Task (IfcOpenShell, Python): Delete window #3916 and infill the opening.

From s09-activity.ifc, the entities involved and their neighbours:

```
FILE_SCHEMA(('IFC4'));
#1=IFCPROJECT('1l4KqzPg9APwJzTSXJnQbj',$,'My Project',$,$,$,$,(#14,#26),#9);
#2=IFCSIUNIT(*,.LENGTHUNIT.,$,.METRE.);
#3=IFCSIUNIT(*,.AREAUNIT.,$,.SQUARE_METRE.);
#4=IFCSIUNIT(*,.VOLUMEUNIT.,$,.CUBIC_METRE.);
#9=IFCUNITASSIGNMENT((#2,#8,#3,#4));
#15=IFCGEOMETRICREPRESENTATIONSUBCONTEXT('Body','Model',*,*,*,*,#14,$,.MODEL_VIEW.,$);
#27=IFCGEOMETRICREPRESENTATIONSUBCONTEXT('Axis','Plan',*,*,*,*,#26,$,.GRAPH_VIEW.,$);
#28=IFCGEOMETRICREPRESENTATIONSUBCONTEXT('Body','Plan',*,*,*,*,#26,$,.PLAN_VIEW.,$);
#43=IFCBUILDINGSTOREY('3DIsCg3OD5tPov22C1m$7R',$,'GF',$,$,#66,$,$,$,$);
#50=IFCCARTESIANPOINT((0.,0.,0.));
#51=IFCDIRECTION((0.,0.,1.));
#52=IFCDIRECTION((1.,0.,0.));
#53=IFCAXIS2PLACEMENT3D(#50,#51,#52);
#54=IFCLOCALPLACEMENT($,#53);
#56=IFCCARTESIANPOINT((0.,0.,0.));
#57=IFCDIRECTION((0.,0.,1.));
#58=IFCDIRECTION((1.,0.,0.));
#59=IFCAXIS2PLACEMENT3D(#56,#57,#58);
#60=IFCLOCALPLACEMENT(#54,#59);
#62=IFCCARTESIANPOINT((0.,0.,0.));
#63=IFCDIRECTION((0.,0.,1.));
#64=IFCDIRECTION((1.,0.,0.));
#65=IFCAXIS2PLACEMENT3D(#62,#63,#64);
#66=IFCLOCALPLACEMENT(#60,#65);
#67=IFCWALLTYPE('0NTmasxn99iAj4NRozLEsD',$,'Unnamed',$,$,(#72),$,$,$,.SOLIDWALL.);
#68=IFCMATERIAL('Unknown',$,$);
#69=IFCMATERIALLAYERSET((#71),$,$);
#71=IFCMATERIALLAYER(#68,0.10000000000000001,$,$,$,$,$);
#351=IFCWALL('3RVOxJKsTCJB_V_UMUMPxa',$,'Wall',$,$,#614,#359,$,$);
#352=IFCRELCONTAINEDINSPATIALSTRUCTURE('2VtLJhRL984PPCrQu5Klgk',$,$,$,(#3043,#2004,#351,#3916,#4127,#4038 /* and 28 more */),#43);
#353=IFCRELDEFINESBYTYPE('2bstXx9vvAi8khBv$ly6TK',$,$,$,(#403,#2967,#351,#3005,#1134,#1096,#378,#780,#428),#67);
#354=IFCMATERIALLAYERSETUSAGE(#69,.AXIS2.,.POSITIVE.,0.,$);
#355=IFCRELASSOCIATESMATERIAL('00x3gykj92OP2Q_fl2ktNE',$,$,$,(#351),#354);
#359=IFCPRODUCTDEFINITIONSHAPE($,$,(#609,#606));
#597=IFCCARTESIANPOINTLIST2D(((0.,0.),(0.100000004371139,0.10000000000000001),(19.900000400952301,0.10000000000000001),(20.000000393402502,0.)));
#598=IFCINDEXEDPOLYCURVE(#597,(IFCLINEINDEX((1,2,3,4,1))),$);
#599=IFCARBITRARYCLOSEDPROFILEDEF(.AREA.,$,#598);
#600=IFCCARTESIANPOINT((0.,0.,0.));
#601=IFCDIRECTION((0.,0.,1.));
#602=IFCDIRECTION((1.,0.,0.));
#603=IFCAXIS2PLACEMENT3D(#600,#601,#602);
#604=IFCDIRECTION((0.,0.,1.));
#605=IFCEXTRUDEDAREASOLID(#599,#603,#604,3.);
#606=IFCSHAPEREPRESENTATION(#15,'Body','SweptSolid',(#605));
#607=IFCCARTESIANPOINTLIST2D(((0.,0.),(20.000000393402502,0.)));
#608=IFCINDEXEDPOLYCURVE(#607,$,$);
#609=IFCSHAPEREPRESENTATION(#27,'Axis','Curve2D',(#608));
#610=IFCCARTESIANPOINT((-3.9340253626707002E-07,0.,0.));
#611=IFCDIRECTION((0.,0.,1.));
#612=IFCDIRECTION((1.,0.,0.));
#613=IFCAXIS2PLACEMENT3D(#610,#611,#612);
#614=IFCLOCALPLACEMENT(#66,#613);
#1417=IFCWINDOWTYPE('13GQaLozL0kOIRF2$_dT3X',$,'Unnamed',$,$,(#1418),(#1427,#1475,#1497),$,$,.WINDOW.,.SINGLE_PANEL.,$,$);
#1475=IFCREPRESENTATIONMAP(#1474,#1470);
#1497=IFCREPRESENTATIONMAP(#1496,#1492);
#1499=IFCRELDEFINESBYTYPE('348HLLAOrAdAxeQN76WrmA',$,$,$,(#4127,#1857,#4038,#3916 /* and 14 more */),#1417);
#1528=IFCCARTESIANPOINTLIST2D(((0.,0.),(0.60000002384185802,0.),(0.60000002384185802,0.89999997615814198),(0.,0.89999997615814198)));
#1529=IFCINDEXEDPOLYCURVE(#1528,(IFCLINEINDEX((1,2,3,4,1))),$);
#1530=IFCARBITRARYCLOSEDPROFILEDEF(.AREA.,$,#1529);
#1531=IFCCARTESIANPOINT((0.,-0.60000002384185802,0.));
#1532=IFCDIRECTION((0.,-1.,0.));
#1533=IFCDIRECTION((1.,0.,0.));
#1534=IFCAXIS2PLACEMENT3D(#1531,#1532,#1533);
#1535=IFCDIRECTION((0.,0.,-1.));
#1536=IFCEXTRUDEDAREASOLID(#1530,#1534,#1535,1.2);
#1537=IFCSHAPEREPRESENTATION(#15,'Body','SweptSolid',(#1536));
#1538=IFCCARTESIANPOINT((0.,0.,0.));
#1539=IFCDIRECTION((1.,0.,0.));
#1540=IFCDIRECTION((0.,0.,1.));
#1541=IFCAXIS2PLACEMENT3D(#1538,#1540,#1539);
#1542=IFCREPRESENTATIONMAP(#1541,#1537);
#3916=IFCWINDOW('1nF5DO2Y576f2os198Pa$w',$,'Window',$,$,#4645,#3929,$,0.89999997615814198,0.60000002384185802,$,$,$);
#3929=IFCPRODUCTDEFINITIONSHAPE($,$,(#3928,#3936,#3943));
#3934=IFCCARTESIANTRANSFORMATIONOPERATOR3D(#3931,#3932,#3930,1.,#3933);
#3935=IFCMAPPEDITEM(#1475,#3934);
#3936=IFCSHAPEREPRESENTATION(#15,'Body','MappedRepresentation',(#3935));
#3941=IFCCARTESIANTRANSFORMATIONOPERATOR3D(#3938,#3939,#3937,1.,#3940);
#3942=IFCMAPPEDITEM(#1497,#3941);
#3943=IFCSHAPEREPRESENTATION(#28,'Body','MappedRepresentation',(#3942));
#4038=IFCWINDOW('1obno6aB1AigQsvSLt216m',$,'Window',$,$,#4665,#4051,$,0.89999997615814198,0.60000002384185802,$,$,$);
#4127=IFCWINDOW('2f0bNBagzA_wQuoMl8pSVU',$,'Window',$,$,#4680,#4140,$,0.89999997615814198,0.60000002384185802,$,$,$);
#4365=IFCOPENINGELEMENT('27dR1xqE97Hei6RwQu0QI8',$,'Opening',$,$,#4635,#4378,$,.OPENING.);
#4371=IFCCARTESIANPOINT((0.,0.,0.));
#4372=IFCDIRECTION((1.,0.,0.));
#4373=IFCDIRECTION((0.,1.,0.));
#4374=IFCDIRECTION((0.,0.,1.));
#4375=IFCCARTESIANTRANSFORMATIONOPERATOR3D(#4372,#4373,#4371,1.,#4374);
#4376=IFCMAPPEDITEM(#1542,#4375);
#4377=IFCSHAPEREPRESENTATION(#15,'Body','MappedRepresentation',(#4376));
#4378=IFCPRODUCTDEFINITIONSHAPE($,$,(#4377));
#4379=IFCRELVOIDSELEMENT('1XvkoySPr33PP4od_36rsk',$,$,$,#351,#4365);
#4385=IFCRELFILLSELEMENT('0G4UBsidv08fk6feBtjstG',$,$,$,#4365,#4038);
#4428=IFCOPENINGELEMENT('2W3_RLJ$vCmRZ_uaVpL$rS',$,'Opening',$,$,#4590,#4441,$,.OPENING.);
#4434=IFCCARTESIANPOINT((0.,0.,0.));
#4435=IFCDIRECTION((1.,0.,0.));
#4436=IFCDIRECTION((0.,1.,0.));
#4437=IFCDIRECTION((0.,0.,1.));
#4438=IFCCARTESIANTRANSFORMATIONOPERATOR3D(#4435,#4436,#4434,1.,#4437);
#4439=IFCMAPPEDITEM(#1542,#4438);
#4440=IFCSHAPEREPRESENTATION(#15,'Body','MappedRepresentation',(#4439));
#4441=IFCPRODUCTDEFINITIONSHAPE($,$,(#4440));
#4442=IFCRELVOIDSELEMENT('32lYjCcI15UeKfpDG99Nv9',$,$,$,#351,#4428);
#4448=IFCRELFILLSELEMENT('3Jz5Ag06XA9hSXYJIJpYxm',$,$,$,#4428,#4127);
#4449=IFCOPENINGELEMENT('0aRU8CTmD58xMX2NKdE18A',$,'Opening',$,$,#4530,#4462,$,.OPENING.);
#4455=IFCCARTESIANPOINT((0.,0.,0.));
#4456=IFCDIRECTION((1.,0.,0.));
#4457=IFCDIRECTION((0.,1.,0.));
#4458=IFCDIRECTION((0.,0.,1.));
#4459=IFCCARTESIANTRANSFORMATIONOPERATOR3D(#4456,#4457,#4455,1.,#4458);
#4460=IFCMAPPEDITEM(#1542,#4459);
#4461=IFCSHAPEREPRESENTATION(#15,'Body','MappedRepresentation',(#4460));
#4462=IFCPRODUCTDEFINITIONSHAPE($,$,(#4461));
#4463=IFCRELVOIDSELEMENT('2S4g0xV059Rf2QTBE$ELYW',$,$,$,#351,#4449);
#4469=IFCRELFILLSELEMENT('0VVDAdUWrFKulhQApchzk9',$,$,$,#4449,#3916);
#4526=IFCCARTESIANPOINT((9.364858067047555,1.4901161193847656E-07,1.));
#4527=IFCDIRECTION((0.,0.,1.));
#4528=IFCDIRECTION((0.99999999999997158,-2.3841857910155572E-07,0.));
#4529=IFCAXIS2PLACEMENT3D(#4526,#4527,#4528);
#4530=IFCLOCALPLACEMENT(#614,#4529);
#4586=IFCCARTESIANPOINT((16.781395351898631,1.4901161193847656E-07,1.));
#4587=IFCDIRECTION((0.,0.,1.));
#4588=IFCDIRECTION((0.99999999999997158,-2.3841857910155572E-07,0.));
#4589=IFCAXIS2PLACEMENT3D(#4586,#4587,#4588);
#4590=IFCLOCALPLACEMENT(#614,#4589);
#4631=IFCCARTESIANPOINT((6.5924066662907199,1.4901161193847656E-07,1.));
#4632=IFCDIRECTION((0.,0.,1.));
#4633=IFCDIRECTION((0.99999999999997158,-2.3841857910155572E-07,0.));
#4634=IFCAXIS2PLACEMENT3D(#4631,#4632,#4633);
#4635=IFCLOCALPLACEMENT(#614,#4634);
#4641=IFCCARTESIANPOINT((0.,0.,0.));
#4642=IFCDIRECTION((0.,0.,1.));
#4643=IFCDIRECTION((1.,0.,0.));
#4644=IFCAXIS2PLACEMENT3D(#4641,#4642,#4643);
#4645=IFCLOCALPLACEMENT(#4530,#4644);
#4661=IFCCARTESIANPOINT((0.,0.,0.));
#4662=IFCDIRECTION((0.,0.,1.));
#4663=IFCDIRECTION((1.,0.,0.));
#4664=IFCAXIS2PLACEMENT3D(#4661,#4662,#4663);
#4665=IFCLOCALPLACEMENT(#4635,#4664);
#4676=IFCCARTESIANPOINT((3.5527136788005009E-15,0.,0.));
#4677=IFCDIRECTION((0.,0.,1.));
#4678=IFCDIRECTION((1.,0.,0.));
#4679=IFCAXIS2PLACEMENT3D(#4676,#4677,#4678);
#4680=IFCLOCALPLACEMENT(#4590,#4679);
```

```python
import ifcopenshell
import ifcopenshell.api.feature
import ifcopenshell.api.root
import ifcopenshell.geom
import ifcopenshell.util.shape

model = ifcopenshell.open("s09-activity.ifc")
settings = ifcopenshell.geom.settings()


def volume(element):
    """Net volume in cubic metres, openings subtracted."""
    shape = ifcopenshell.geom.create_shape(settings, element)
    return ifcopenshell.util.shape.get_volume(shape.geometry)


window = model.by_guid("1nF5DO2Y576f2os198Pa$w")
opening = window.FillsVoids[0].RelatingOpeningElement
wall = opening.VoidsElements[0].RelatingBuildingElement
before = volume(wall)

ifcopenshell.api.root.remove_product(model, product=window)
ifcopenshell.api.feature.remove_feature(model, feature=opening)

after = volume(wall)

print(f"wall volume {before:.3f} -> {after:.3f} m3")

model.write("s09-activity_updated.ifc")
```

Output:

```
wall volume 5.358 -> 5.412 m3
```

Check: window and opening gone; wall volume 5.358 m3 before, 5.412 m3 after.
